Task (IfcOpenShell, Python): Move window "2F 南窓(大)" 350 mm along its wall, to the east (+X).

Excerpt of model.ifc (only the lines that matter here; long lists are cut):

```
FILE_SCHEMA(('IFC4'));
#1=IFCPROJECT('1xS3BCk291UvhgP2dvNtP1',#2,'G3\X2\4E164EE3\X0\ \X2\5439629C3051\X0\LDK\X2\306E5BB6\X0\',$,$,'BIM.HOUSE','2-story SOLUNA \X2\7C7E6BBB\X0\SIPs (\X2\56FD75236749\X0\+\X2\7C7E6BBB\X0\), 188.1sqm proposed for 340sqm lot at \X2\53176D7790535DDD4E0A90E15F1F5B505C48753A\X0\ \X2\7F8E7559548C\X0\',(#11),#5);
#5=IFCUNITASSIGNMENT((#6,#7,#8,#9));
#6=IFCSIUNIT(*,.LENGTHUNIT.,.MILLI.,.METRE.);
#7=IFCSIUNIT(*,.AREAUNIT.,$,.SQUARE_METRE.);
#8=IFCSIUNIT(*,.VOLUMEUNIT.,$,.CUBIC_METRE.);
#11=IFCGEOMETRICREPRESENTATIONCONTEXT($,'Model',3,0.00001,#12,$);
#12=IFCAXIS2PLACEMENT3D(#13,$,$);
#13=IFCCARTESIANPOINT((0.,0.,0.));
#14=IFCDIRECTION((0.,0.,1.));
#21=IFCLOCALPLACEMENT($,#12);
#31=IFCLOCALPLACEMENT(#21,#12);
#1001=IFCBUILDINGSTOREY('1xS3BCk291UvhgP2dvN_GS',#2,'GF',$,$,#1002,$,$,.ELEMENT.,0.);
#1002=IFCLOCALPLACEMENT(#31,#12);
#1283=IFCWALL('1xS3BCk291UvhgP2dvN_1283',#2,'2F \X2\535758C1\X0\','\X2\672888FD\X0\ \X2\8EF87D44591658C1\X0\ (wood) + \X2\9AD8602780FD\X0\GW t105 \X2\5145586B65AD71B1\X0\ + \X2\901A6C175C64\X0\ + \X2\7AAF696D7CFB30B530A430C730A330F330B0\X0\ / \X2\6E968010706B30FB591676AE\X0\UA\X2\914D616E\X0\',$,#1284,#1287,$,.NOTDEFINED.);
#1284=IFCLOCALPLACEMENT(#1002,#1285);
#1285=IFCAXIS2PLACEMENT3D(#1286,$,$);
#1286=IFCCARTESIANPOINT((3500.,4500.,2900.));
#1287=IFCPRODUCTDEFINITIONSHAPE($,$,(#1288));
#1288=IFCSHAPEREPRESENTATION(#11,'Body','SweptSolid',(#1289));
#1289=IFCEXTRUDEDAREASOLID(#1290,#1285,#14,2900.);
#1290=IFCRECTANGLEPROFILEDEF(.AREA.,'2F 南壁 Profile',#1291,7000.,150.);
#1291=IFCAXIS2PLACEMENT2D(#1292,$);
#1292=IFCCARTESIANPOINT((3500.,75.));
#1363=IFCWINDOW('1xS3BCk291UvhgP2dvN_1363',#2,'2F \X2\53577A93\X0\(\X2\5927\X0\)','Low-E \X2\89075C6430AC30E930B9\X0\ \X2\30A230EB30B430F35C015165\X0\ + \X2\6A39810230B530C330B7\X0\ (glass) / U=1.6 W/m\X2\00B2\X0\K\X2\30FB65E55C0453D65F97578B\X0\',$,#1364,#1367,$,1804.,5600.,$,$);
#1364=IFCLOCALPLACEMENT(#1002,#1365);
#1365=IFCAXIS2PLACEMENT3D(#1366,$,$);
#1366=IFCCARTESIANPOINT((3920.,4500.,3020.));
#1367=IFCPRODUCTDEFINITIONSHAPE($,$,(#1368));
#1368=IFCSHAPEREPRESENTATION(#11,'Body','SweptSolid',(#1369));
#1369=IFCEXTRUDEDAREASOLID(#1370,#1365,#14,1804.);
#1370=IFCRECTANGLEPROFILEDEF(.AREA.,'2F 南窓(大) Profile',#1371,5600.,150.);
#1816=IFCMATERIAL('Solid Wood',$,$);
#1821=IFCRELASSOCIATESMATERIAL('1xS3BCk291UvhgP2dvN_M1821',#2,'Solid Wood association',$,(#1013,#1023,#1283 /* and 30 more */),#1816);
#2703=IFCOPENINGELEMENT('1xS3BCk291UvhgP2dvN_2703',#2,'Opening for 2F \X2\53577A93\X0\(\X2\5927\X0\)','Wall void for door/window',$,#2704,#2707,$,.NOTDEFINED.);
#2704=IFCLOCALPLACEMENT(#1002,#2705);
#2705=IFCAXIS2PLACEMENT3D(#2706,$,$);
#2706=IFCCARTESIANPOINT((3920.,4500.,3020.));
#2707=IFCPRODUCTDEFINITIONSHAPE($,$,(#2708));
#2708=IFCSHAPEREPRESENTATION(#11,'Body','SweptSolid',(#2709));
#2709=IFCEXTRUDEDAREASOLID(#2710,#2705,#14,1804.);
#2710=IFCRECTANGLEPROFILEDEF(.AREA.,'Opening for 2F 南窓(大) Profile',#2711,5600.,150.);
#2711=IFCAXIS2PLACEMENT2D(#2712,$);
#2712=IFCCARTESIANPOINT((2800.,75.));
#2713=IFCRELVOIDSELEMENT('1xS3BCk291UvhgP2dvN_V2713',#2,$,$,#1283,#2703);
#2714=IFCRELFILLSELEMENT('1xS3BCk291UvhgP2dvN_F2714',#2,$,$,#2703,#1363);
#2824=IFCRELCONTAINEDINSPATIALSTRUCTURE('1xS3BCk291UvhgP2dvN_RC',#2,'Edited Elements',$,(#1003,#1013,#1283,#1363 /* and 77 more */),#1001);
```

```python
import ifcopenshell
import ifcopenshell.api.geometry
import ifcopenshell.util.placement

model = ifcopenshell.open("model.ifc")

window = model.by_guid("1xS3BCk291UvhgP2dvN_1363")
opening = window.FillsVoids[0].RelatingOpeningElement
wall = opening.VoidsElements[0].RelatingBuildingElement

wall_matrix = ifcopenshell.util.placement.get_local_placement(wall.ObjectPlacement)
shift = wall_matrix[:3, 0] * 350.0
before = ifcopenshell.util.placement.get_local_placement(window.ObjectPlacement)[:3, 3].copy()

# The window is not placed relative to its opening, so move both.
for product in (opening, window):
    matrix = ifcopenshell.util.placement.get_local_placement(product.ObjectPlacement)
    matrix[:3, 3] += shift
    ifcopenshell.api.geometry.edit_object_placement(model, product=product, matrix=matrix, is_si=False)

after = ifcopenshell.util.placement.get_local_placement(window.ObjectPlacement)[:3, 3]
print("window moved by", (after - before).round(3) + 0.0)

model.write("model_edited.ifc")
```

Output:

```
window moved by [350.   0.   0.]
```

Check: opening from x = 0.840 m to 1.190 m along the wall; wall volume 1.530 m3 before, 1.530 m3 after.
